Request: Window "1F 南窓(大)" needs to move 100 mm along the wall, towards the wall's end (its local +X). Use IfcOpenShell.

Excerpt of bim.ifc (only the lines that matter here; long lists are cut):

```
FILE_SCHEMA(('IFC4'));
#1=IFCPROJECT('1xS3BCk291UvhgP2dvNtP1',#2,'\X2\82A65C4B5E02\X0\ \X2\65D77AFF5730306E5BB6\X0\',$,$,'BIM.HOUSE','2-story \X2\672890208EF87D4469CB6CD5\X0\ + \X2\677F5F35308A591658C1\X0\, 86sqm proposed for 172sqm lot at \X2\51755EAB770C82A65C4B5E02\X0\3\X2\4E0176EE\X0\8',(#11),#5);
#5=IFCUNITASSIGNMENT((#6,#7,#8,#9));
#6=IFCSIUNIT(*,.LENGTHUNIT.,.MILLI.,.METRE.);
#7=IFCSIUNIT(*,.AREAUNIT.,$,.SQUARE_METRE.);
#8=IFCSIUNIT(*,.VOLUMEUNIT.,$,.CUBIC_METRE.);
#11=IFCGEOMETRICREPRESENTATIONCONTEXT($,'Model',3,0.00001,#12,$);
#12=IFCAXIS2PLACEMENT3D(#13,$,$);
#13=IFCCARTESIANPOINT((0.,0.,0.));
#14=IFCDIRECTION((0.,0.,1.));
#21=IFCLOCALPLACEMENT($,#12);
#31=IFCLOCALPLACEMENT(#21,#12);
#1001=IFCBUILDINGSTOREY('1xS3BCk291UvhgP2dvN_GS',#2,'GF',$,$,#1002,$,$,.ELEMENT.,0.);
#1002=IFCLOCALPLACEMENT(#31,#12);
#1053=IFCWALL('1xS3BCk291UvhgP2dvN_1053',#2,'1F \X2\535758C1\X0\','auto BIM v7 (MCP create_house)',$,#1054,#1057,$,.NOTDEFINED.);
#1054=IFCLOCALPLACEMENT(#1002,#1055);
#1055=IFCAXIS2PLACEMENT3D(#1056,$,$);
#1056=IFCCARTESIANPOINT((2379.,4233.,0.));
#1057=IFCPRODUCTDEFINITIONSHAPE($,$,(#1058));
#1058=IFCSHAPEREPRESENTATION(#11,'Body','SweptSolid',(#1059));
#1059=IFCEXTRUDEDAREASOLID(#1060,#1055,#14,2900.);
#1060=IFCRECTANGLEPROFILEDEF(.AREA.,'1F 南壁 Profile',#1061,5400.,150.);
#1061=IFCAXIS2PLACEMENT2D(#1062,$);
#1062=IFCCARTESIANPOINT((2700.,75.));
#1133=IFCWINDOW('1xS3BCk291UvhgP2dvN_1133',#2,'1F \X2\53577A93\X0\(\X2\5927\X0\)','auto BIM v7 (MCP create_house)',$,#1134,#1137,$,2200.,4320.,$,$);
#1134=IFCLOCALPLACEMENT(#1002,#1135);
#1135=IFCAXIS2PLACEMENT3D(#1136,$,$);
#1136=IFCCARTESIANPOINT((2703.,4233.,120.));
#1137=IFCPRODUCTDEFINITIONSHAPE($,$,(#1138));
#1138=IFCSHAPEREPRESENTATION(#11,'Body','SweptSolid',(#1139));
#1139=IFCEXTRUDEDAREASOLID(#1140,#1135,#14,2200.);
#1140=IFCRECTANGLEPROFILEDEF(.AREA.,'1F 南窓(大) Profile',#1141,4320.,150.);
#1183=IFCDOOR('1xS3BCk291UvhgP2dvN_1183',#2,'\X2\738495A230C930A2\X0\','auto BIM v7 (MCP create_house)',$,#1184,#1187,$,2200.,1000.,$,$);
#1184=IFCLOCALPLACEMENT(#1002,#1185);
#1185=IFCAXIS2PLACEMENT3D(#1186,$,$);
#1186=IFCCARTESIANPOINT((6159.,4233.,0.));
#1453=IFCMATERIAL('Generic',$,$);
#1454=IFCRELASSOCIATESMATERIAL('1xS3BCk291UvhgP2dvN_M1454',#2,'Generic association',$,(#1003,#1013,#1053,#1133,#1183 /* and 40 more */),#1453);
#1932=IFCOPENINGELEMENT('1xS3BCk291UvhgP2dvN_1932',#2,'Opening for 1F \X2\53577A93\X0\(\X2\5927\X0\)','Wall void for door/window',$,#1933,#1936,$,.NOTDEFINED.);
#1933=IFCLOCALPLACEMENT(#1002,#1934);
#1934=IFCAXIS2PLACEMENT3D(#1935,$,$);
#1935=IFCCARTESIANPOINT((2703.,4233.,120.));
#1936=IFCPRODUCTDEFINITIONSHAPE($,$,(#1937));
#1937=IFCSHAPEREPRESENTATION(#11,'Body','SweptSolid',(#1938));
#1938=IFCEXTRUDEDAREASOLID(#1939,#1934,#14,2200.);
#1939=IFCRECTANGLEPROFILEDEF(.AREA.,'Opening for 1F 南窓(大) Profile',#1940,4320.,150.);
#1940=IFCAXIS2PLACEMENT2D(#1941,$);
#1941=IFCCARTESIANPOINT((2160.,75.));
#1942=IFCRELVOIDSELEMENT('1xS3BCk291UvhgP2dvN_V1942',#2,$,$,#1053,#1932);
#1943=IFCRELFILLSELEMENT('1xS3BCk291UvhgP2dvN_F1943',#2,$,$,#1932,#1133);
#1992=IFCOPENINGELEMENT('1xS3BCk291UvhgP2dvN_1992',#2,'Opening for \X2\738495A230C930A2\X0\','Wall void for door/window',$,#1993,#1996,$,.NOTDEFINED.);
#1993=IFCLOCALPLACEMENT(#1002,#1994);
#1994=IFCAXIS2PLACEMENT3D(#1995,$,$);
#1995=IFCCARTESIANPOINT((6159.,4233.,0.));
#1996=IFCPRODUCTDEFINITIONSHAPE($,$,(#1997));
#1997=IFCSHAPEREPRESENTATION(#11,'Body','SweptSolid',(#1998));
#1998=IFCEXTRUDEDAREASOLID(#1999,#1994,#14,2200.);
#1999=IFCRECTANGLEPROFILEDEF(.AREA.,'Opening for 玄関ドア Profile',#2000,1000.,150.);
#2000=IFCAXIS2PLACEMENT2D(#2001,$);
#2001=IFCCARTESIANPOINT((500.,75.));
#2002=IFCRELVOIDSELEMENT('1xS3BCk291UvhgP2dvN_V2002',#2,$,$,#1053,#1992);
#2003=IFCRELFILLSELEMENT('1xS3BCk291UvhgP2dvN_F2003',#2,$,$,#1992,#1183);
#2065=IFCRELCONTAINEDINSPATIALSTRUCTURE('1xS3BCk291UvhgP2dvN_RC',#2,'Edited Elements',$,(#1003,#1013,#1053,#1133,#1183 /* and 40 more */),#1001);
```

```python
import ifcopenshell
import ifcopenshell.api.geometry
import ifcopenshell.util.placement
import ifcopenshell.util.unit

model = ifcopenshell.open("bim.ifc")
unit_scale = ifcopenshell.util.unit.calculate_unit_scale(model)

window = model.by_guid("1xS3BCk291UvhgP2dvN_1133")
opening = window.FillsVoids[0].RelatingOpeningElement
wall = opening.VoidsElements[0].RelatingBuildingElement

wall_matrix = ifcopenshell.util.placement.get_local_placement(wall.ObjectPlacement)
shift = wall_matrix[:3, 0] * 0.1 / unit_scale
before = ifcopenshell.util.placement.get_local_placement(window.ObjectPlacement)[:3, 3].copy()

# The window is not placed relative to its opening, so move both.
for product in (opening, window):
    matrix = ifcopenshell.util.placement.get_local_placement(product.ObjectPlacement)
    matrix[:3, 3] += shift
    ifcopenshell.api.geometry.edit_object_placement(model, product=product, matrix=matrix, is_si=False)

after = ifcopenshell.util.placement.get_local_placement(window.ObjectPlacement)[:3, 3]
print("window moved by", (after - before).round(3) + 0.0)

model.write("bim_v2.ifc")
```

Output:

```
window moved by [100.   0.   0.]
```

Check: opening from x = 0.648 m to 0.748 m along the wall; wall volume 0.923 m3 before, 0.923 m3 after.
